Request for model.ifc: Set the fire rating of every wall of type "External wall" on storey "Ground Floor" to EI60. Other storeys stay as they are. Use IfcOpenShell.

First a look at what the model holds.

```python
import ifcopenshell
import ifcopenshell.util.element

model = ifcopenshell.open("model.ifc")
print(model.schema)
storey = next(s for s in model.by_type("IfcBuildingStorey") if s.Name == "Ground Floor")
walls = [e for e in ifcopenshell.util.element.get_decomposition(storey) if e.is_a("IfcWall")]
seen = {}
for e in walls:
    element_type = ifcopenshell.util.element.get_type(e)
    key = (element_type.Name if element_type != e and element_type else None, ifcopenshell.util.element.get_pset(e, "Pset_WallCommon", "FireRating"))
    seen[key] = seen.get(key, 0) + 1
for (name, value), count in sorted(seen.items(), key=str):
    print(count, "x", name, "|", value)
```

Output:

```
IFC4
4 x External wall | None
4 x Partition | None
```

```python
import ifcopenshell
import ifcopenshell.api.pset
import ifcopenshell.util.element

model = ifcopenshell.open("model.ifc")

storey = next(s for s in model.by_type("IfcBuildingStorey") if s.Name == "Ground Floor")
walls = [e for e in ifcopenshell.util.element.get_decomposition(storey) if e.is_a("IfcWall")]

count = 0
for e in walls:
    element_type = ifcopenshell.util.element.get_type(e)
    if element_type in (None, e) or element_type.Name != "External wall":
        continue
    # add_pset returns the element's existing set when there is one.
    pset = ifcopenshell.api.pset.add_pset(model, product=e, name="Pset_WallCommon")
    ifcopenshell.api.pset.edit_pset(model, pset=pset, properties={"FireRating": "EI60"})
    count += 1

print(count, "walls updated")

model.write("model_updated.ifc")
```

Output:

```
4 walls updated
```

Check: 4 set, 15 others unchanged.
